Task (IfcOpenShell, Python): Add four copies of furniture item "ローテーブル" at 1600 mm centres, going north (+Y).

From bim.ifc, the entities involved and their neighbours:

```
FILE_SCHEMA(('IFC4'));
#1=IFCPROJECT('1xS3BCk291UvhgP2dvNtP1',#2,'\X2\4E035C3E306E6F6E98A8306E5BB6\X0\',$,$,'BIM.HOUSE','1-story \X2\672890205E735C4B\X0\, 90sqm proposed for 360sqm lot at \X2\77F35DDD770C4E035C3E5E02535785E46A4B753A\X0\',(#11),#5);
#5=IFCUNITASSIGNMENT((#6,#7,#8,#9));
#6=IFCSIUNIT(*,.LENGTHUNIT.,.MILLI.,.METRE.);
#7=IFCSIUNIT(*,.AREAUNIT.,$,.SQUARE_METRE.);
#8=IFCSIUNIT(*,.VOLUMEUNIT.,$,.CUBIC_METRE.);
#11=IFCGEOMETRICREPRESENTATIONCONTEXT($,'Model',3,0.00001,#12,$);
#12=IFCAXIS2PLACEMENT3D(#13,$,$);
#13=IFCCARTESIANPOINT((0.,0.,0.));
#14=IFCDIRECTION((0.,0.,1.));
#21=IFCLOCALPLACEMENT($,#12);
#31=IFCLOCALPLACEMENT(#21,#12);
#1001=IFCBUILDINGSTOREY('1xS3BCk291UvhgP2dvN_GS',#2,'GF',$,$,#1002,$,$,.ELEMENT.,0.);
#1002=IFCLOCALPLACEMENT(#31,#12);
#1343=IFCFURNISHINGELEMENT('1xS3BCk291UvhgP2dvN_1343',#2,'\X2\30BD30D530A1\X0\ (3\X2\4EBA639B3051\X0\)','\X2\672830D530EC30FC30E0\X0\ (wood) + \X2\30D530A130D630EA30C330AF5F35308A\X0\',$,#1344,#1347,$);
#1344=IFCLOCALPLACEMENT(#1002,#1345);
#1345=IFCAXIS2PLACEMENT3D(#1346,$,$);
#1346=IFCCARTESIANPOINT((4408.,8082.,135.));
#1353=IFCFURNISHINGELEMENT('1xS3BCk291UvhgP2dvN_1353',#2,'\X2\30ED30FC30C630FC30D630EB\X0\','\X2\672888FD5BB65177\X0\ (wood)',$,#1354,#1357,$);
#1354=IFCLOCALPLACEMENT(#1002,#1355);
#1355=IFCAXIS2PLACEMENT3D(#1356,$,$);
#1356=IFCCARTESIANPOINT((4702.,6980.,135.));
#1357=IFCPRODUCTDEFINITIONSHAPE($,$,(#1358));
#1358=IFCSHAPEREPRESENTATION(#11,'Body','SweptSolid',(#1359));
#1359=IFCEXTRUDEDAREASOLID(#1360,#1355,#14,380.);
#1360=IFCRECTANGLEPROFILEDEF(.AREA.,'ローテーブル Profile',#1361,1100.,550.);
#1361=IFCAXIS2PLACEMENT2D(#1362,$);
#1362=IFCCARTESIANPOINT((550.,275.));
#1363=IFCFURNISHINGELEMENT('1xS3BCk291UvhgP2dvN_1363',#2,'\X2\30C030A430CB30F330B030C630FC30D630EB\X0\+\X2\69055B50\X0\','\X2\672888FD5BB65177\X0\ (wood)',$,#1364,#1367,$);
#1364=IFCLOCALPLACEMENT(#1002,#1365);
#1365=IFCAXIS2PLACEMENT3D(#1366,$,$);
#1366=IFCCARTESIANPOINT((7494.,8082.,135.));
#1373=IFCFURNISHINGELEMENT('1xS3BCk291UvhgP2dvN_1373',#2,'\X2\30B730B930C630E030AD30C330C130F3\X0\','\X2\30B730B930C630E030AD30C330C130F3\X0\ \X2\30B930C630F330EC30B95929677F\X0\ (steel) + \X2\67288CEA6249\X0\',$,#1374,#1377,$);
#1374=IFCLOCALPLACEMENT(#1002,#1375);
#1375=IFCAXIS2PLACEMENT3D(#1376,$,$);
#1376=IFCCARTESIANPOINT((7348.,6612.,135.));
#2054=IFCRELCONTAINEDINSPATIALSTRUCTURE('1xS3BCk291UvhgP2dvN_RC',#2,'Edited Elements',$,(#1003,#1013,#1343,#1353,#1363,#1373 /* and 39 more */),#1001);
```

```python
import numpy as np
import ifcopenshell
import ifcopenshell.api.geometry
import ifcopenshell.api.root
import ifcopenshell.util.element
import ifcopenshell.util.placement

model = ifcopenshell.open("bim.ifc")


def reuse_history(source, copy):
    """copy_class also copies each property set's owner history, people and application; keep the originals."""
    for rel in copy.IsDefinedBy:
        if rel.is_a("IfcRelDefinesByProperties") and (history := rel.RelatingPropertyDefinition.OwnerHistory):
            rel.RelatingPropertyDefinition.OwnerHistory = source.OwnerHistory
            ifcopenshell.util.element.remove_deep2(model, history)


source = model.by_guid("1xS3BCk291UvhgP2dvN_1353")
base = ifcopenshell.util.placement.get_local_placement(source.ObjectPlacement)
step = np.array([0.0, 1.0, 0.0]) * 1600.0

for i in range(1, 5):
    copy = ifcopenshell.api.root.copy_class(model, product=source)
    copy.Representation = ifcopenshell.util.element.copy_deep(
        model, source.Representation, exclude=["IfcGeometricRepresentationContext", "IfcRepresentationMap"]
    )
    reuse_history(source, copy)
    matrix = base.copy()
    matrix[:3, 3] += i * step
    print("added at", matrix[:3, 3].round(3) + 0.0)
    ifcopenshell.api.geometry.edit_object_placement(model, product=copy, matrix=matrix, is_si=False)

model.write("bim_edited.ifc")
```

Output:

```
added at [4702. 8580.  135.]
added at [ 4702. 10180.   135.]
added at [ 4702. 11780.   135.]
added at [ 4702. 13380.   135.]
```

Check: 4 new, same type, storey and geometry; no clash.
